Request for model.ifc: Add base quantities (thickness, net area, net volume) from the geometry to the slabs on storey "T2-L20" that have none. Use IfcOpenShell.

First a look at what the model holds.

```python
import ifcopenshell
import ifcopenshell.util.element
import ifcopenshell.util.unit

model = ifcopenshell.open("model.ifc")
print(model.schema)
for unit_type in ("LENGTHUNIT", "AREAUNIT", "VOLUMEUNIT"):
    print(unit_type, ifcopenshell.util.unit.calculate_unit_scale(model, unit_type))
storey = next(s for s in model.by_type("IfcBuildingStorey") if s.Name == "T2-L20")
slabs = [e for e in ifcopenshell.util.element.get_decomposition(storey) if e.is_a("IfcSlab")]
for e in sorted(slabs, key=lambda e: e.id()):
    print(e.id(), e.is_a(), e.Name, list(ifcopenshell.util.element.get_psets(e, qtos_only=True)), sep=" | ")
```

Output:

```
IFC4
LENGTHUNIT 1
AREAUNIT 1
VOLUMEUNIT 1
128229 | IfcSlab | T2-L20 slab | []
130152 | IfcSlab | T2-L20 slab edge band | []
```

```python
import ifcopenshell
import ifcopenshell.api.pset
import ifcopenshell.geom
import ifcopenshell.util.element
import ifcopenshell.util.shape
import ifcopenshell.util.unit

model = ifcopenshell.open("model.ifc")
unit_scale = ifcopenshell.util.unit.calculate_unit_scale(model)
area_scale = ifcopenshell.util.unit.calculate_unit_scale(model, "AREAUNIT")
volume_scale = ifcopenshell.util.unit.calculate_unit_scale(model, "VOLUMEUNIT")
settings = ifcopenshell.geom.settings()

storey = next(s for s in model.by_type("IfcBuildingStorey") if s.Name == "T2-L20")
slabs = [e for e in ifcopenshell.util.element.get_decomposition(storey) if e.is_a("IfcSlab")]

for e in sorted(slabs, key=lambda e: e.id()):
    if ifcopenshell.util.element.get_psets(e, qtos_only=True, should_inherit=False):
        continue
    # Geometry comes back in metres, in the element's own axes.
    shape = ifcopenshell.geom.create_shape(settings, e)
    values = {
        "Width": ifcopenshell.util.shape.get_z(shape.geometry) / unit_scale,
        "NetArea": ifcopenshell.util.shape.get_footprint_area(shape.geometry) / area_scale,
        "NetVolume": ifcopenshell.util.shape.get_volume(shape.geometry) / volume_scale,
    }
    qto = ifcopenshell.api.pset.add_qto(model, product=e, name="Qto_SlabBaseQuantities")
    ifcopenshell.api.pset.edit_qto(model, qto=qto, properties=values)
    print(e.id(), {k: round(v, 3) for k, v in values.items()})

model.write("model_rev.ifc")
```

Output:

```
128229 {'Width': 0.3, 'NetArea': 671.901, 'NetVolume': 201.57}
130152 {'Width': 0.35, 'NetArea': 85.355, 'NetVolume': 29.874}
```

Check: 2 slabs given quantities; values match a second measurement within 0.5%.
